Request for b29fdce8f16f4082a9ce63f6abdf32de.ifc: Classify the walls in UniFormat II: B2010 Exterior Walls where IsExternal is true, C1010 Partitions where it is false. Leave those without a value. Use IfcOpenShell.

First a look at what the model holds.

```python
import ifcopenshell
import ifcopenshell.util.element

model = ifcopenshell.open("b29fdce8f16f4082a9ce63f6abdf32de.ifc")
print(model.schema)
print("classifications:", [c.Name for c in model.by_type("IfcClassification")])
values = [ifcopenshell.util.element.get_pset(e, "Pset_WallCommon", "IsExternal") for e in model.by_type("IfcWall")]
for value in (True, False, None):
    print("IsExternal", value, values.count(value))
```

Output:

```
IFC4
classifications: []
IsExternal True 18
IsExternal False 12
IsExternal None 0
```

```python
import ifcopenshell
import ifcopenshell.api.classification
import ifcopenshell.util.element

model = ifcopenshell.open("b29fdce8f16f4082a9ce63f6abdf32de.ifc")

system = ifcopenshell.api.classification.add_classification(model, classification="UniFormat II")

walls = model.by_type("IfcWall")
external = {e: ifcopenshell.util.element.get_pset(e, "Pset_WallCommon", "IsExternal") for e in walls}
for flag, code, name in ((True, "B2010", "Exterior Walls"), (False, "C1010", "Partitions")):
    products = [e for e in walls if external[e] is flag]
    ifcopenshell.api.classification.add_reference(
        model, products=products, classification=system, identification=code, name=name
    )
    print(code, len(products))

model.write("b29fdce8f16f4082a9ce63f6abdf32de_edited.ifc")
```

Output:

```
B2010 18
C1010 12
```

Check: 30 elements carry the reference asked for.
